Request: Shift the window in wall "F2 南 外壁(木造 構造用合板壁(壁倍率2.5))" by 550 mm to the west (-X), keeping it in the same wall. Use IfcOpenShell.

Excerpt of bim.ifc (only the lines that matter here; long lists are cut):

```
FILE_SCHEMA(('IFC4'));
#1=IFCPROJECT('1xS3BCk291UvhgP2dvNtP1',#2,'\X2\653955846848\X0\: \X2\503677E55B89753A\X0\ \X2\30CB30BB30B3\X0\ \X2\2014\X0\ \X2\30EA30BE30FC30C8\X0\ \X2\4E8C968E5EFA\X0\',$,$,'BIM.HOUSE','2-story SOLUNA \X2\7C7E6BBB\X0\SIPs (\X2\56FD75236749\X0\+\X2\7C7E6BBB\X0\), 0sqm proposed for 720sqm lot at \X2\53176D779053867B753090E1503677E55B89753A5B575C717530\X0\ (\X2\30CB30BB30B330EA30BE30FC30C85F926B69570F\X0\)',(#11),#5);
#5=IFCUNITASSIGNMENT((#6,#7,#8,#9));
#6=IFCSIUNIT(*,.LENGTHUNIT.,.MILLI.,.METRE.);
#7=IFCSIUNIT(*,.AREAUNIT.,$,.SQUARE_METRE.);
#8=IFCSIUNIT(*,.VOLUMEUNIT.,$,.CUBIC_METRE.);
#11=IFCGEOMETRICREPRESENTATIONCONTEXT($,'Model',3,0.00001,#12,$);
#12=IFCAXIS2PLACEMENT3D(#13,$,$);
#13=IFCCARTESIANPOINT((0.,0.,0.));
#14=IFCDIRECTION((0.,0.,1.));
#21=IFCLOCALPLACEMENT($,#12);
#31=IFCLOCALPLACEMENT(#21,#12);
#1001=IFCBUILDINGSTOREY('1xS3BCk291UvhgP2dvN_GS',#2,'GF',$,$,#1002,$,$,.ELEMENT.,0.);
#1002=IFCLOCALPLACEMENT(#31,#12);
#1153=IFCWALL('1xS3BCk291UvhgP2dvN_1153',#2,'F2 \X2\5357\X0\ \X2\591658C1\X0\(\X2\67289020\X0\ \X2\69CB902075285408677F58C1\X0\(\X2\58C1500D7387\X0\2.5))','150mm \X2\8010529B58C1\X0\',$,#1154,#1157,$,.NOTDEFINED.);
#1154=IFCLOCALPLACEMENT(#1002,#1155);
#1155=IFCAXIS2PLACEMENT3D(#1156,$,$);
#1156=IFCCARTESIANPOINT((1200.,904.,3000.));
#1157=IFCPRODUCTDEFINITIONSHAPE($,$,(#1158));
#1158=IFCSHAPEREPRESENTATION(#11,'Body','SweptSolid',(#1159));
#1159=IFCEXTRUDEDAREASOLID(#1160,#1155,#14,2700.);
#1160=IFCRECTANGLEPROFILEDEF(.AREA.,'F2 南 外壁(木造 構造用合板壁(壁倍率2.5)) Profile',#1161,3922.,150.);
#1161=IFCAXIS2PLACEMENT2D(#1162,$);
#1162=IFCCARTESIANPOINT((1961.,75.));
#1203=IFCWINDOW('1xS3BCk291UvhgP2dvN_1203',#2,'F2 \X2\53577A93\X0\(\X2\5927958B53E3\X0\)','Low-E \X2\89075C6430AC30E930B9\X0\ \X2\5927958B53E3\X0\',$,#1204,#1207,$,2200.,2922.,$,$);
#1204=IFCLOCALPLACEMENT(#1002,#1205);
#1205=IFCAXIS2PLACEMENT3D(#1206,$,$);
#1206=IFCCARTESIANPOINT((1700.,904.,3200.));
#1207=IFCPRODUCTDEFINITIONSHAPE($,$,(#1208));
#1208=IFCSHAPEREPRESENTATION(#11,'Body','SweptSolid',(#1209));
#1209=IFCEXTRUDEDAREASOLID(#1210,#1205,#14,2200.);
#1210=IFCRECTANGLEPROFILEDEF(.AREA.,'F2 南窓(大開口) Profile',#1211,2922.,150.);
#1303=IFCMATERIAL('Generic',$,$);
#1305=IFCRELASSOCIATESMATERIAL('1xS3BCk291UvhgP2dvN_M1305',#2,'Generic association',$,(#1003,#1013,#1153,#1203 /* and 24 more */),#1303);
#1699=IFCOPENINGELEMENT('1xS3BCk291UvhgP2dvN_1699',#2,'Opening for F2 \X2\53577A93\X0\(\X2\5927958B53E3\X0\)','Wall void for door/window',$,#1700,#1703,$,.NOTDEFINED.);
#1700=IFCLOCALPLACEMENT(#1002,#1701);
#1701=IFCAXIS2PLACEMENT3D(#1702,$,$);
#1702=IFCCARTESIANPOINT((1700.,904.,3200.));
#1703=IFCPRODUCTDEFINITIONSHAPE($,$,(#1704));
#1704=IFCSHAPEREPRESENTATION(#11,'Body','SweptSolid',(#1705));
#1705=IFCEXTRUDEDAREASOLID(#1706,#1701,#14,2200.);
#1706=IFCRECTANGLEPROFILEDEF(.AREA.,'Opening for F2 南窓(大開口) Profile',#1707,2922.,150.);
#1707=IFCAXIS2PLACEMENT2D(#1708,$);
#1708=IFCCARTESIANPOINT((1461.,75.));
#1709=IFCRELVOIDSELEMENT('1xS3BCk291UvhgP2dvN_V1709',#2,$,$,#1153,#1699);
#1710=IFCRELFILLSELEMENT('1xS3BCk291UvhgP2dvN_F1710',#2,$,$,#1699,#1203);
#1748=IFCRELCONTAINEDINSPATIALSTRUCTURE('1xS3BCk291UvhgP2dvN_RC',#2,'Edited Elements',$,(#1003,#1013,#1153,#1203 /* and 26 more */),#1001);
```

```python
import ifcopenshell
import ifcopenshell.api.geometry
import ifcopenshell.util.placement
import ifcopenshell.util.unit

model = ifcopenshell.open("bim.ifc")
unit_scale = ifcopenshell.util.unit.calculate_unit_scale(model)

window = model.by_guid("1xS3BCk291UvhgP2dvN_1203")
opening = window.FillsVoids[0].RelatingOpeningElement
wall = opening.VoidsElements[0].RelatingBuildingElement

wall_matrix = ifcopenshell.util.placement.get_local_placement(wall.ObjectPlacement)
shift = wall_matrix[:3, 0] * -0.55 / unit_scale
before = ifcopenshell.util.placement.get_local_placement(window.ObjectPlacement)[:3, 3].copy()

# The window is not placed relative to its opening, so move both.
for product in (opening, window):
    matrix = ifcopenshell.util.placement.get_local_placement(product.ObjectPlacement)
    matrix[:3, 3] += shift
    ifcopenshell.api.geometry.edit_object_placement(model, product=product, matrix=matrix, is_si=False)

after = ifcopenshell.util.placement.get_local_placement(window.ObjectPlacement)[:3, 3]
print("window moved by", (after - before).round(3) + 0.0)

model.write("bim_rev.ifc")
```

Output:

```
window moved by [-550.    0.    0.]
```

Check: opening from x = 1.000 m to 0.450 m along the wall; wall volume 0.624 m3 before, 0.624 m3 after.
